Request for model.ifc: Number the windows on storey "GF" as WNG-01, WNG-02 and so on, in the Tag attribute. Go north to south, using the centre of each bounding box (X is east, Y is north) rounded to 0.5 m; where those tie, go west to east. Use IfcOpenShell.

First a look at what the model holds.

```python
import ifcopenshell
import ifcopenshell.util.element
import ifcopenshell.util.placement

model = ifcopenshell.open("model.ifc")
print(model.schema)
storey = next(s for s in model.by_type("IfcBuildingStorey") if s.Name == "GF")
windows = [e for e in ifcopenshell.util.element.get_decomposition(storey) if e.is_a("IfcWindow")]
for e in sorted(windows, key=lambda e: e.id()):
    origin = ifcopenshell.util.placement.get_local_placement(e.ObjectPlacement)[:3, 3]
    print(e.id(), e.Tag, e.Name, origin.round(2) + 0.0, sep=" | ")
```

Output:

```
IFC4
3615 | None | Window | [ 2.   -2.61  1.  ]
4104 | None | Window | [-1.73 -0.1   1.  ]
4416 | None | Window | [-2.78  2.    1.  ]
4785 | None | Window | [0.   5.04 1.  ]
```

```python
import ifcopenshell
import ifcopenshell.geom
import ifcopenshell.util.element
import ifcopenshell.util.shape

model = ifcopenshell.open("model.ifc")
settings = ifcopenshell.geom.settings()
settings.set("use-world-coords", True)


def centre(element):
    shape = ifcopenshell.geom.create_shape(settings, element)
    return ifcopenshell.util.shape.get_bbox_centroid(shape.geometry)


storey = next(s for s in model.by_type("IfcBuildingStorey") if s.Name == "GF")
windows = [e for e in ifcopenshell.util.element.get_decomposition(storey) if e.is_a("IfcWindow")]

# Insertion points can sit at a corner or the storey origin, so sort by the geometry (in metres).
centres = {e: centre(e) for e in windows}
windows.sort(key=lambda e: (-round(centres[e][1] / 0.5), centres[e][0]))

for i, e in enumerate(windows, start=1):
    number = f"WNG-{i:02d}"
    e.Tag = number
    print(e.id(), number)

model.write("model_rev.ifc")
```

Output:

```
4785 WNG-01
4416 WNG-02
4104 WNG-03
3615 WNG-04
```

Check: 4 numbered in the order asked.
